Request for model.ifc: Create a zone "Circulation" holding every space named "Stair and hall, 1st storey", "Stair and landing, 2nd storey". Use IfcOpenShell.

First a look at what the model holds.

```python
import ifcopenshell

model = ifcopenshell.open("model.ifc")
print(model.schema)
seen = {}
for space in model.by_type("IfcSpace"):
    seen[space.LongName] = seen.get(space.LongName, 0) + 1
for name, count in sorted(seen.items(), key=str):
    print(count, "x", name)
print("zones:", [z.Name for z in model.by_type("IfcZone")][:20])
```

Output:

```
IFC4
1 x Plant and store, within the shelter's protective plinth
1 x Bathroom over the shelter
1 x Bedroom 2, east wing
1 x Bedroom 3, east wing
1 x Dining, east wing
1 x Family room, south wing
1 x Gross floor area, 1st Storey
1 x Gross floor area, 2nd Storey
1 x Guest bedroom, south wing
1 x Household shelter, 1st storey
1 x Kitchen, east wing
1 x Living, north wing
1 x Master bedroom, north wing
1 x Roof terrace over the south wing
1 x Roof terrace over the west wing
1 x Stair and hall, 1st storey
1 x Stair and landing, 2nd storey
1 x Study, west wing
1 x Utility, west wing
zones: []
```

```python
import ifcopenshell
import ifcopenshell.api.group
import ifcopenshell.api.root

model = ifcopenshell.open("model.ifc")

names = {"Stair and hall, 1st storey", "Stair and landing, 2nd storey"}
spaces = [s for s in model.by_type("IfcSpace") if s.LongName in names]

zone = ifcopenshell.api.root.create_entity(model, ifc_class="IfcZone", name="Circulation")
ifcopenshell.api.group.assign_group(model, products=spaces, group=zone)
print(len(spaces), "spaces in", zone.Name)

model.write("model_rev.ifc")
```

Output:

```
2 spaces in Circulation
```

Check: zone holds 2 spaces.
